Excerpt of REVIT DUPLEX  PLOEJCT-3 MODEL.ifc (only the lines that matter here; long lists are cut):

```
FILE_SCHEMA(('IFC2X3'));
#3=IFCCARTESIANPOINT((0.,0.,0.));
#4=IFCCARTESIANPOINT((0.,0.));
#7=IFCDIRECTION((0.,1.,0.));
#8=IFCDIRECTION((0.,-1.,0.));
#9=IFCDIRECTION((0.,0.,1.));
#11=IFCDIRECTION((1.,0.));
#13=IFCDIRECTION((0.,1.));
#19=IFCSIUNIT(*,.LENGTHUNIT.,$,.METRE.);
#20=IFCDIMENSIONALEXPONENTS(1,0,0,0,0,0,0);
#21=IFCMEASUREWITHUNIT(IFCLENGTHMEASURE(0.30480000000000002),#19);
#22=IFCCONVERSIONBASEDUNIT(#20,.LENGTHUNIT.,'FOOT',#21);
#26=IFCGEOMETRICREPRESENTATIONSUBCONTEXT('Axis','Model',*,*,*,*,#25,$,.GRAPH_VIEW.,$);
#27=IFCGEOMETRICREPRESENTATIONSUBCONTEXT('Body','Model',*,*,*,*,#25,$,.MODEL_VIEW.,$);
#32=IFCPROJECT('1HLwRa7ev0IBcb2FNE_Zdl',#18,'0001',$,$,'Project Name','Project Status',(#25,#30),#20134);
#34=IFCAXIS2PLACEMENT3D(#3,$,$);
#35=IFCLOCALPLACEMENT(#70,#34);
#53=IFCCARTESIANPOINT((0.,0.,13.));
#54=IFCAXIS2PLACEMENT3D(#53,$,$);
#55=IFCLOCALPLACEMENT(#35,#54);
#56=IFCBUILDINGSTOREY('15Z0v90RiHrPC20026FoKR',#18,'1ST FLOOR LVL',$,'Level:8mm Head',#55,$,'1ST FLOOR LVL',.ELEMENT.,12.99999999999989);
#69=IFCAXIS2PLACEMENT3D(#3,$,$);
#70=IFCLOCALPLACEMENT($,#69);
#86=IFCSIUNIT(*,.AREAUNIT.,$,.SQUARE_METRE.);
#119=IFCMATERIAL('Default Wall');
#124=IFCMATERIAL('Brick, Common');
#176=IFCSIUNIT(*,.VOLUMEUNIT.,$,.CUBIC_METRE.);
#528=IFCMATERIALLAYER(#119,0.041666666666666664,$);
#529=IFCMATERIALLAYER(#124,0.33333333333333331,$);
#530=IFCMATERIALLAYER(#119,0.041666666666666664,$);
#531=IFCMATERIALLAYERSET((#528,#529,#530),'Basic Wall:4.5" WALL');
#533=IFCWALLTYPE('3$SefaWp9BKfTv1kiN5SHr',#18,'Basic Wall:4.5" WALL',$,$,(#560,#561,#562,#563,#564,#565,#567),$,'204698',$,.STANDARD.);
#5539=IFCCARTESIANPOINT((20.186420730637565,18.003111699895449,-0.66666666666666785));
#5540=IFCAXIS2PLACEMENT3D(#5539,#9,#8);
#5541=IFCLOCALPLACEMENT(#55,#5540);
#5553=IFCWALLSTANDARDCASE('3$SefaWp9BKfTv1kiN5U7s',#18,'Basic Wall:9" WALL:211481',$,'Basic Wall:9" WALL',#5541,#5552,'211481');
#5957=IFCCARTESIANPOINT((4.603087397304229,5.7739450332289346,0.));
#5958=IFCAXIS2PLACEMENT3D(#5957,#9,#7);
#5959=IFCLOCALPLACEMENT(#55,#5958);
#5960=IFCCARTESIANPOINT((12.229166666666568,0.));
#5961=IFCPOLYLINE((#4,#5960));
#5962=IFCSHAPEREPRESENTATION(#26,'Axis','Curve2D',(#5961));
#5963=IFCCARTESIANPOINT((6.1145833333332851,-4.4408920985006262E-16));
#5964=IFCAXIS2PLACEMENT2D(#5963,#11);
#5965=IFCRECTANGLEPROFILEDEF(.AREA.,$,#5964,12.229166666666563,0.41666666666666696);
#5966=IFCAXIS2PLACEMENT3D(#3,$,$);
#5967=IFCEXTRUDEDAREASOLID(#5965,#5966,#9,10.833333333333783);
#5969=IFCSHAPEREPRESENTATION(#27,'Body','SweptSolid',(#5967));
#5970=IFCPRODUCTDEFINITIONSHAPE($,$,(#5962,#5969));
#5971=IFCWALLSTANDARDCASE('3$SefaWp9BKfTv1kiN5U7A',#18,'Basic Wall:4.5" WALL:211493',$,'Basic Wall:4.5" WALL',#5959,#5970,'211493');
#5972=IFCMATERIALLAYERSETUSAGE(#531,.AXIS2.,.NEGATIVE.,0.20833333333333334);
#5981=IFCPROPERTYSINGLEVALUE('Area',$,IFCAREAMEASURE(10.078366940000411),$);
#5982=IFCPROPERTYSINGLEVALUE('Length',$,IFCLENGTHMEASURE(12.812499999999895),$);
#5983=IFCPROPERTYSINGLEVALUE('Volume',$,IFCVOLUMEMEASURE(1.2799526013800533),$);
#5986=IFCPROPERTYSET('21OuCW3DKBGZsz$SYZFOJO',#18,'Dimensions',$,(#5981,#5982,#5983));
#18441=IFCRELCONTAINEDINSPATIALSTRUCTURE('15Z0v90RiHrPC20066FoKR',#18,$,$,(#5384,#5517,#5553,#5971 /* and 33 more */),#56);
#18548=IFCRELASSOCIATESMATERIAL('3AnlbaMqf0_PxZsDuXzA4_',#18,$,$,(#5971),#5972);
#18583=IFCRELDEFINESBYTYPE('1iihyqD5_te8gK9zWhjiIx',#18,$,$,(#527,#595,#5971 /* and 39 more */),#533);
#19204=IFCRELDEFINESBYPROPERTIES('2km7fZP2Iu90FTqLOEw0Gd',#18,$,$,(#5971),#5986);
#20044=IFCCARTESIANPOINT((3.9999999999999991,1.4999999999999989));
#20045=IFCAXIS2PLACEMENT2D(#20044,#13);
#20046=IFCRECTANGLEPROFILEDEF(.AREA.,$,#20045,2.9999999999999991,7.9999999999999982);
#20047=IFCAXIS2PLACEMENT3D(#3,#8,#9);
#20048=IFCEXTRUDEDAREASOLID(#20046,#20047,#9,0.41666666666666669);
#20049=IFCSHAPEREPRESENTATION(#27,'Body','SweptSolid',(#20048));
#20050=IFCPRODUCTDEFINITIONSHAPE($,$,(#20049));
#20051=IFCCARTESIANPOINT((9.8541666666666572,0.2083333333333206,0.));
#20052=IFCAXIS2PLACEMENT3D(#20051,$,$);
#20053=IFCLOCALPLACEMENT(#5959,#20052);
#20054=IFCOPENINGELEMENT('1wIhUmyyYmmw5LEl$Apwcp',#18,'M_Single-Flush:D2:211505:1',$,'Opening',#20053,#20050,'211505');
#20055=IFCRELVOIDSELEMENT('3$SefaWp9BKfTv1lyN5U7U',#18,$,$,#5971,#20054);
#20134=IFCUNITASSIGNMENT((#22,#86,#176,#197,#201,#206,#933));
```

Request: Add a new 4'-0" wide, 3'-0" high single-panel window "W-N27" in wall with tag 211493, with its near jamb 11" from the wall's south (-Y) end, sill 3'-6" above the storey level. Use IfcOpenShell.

```python
import numpy as np
import ifcopenshell
import ifcopenshell.api.feature
import ifcopenshell.api.geometry
import ifcopenshell.api.pset
import ifcopenshell.api.root
import ifcopenshell.api.spatial
import ifcopenshell.api.type
import ifcopenshell.geom
import ifcopenshell.util.element
import ifcopenshell.util.placement
import ifcopenshell.util.representation
import ifcopenshell.util.shape
import ifcopenshell.util.unit

model = ifcopenshell.open("REVIT DUPLEX  PLOEJCT-3 MODEL.ifc")
unit_scale = ifcopenshell.util.unit.calculate_unit_scale(model)
area_scale = ifcopenshell.util.unit.calculate_unit_scale(model, "AREAUNIT")
volume_scale = ifcopenshell.util.unit.calculate_unit_scale(model, "VOLUMEUNIT")
settings = ifcopenshell.geom.settings()


def volume(element):
    """Net volume in cubic metres, openings subtracted."""
    shape = ifcopenshell.geom.create_shape(settings, element)
    return ifcopenshell.util.shape.get_volume(shape.geometry)


wall = model.by_guid("3$SefaWp9BKfTv1kiN5U7A")
storey = ifcopenshell.util.element.get_container(wall, ifc_class="IfcBuildingStorey")
context = ifcopenshell.util.representation.get_context(model, "Model", "Body", "MODEL_VIEW")
before = volume(wall)

width, height, from_end, sill = 1.2192, 0.9144, 0.2794, 1.0668  # metres

# The wall runs along its own X axis, and the end named is its -X end.
wall_shape = ifcopenshell.geom.create_shape(settings, wall)
x, y, z = ifcopenshell.util.shape.get_vertices(wall_shape.geometry).T
start = x.min() + from_end
face, thickness = float(y.min()), float(y.max() - y.min())
wall_matrix = ifcopenshell.util.placement.get_local_placement(wall.ObjectPlacement)
level = ifcopenshell.util.placement.get_local_placement(storey.ObjectPlacement)[2, 3]


def in_wall(x, y):
    """Placement at x, y metres in the wall's axes, at sill height."""
    matrix = wall_matrix.copy()
    matrix[:, 3] = wall_matrix @ np.array([x / unit_scale, y / unit_scale, 0.0, 1.0])
    matrix[2, 3] = level + sill / unit_scale
    return matrix


# Opening: a box that overshoots both wall faces by 50 mm.
opening = ifcopenshell.api.root.create_entity(model, ifc_class="IfcOpeningElement")
box = ifcopenshell.api.geometry.add_wall_representation(
    model, context=context, length=width, height=height, thickness=thickness + 0.1
)
ifcopenshell.api.geometry.assign_representation(model, product=opening, representation=box)
ifcopenshell.api.geometry.edit_object_placement(model, product=opening, matrix=in_wall(start, face - 0.05), is_si=False)
ifcopenshell.api.feature.add_feature(model, feature=opening, element=wall)

window = ifcopenshell.api.root.create_entity(model, ifc_class="IfcWindow", name="W-N27")
window.OverallWidth, window.OverallHeight = width / unit_scale, height / unit_scale
body = ifcopenshell.api.geometry.add_window_representation(
    model,
    context=context,
    overall_width=window.OverallWidth,
    overall_height=window.OverallHeight,
    partition_type="SINGLE_PANEL",
)
ifcopenshell.api.geometry.assign_representation(model, product=window, representation=body)
ifcopenshell.api.spatial.assign_container(model, products=[window], relating_structure=storey)
fills = ifcopenshell.api.feature.add_filling(model, opening=opening, element=window)
fills.OwnerHistory = window.OwnerHistory  # required in IFC2X3

# IFC2X3 keeps the operation on the window style.
style = ifcopenshell.api.root.create_entity(model, ifc_class="IfcWindowStyle", name="W-N27")
style.OperationType, style.ConstructionType = "SINGLE_PANEL", "NOTDEFINED"
style.ParameterTakesPrecedence = style.Sizeable = False
ifcopenshell.api.type.assign_type(model, related_objects=[window], relating_type=style)

# Centre the window in the wall's thickness.
ifcopenshell.api.geometry.edit_object_placement(model, product=window, matrix=in_wall(start, face), is_si=False)
window_shape = ifcopenshell.geom.create_shape(settings, window)
depth = ifcopenshell.util.shape.get_vertices(window_shape.geometry)[:, 1]
offset = face + thickness / 2 - (depth.min() + depth.max()) / 2
ifcopenshell.api.geometry.edit_object_placement(model, product=window, matrix=in_wall(start, offset), is_si=False)

after = volume(wall)

# Update the wall's stored quantities.
pset = model.by_id(ifcopenshell.util.element.get_pset(wall, "Dimensions", should_inherit=False)["id"])
ifcopenshell.api.pset.edit_pset(model, pset=pset, properties={
    "Area": model.create_entity("IfcAreaMeasure", after / thickness / area_scale),
    "Volume": model.create_entity("IfcVolumeMeasure", after / volume_scale),
})

print(f"wall volume {before:.3f} -> {after:.3f} m3")

model.write("REVIT DUPLEX  PLOEJCT-3 MODEL_edited.ifc")
```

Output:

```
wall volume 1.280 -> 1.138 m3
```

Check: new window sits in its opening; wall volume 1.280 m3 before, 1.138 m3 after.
